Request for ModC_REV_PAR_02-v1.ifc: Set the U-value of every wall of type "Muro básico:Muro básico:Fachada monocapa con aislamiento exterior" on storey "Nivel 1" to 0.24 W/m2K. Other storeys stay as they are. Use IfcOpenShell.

First a look at what the model holds.

```python
import ifcopenshell
import ifcopenshell.util.element

model = ifcopenshell.open("ModC_REV_PAR_02-v1.ifc")
print(model.schema)
storey = next(s for s in model.by_type("IfcBuildingStorey") if s.Name == "Nivel 1")
walls = [e for e in ifcopenshell.util.element.get_decomposition(storey) if e.is_a("IfcWall")]
seen = {}
for e in walls:
    element_type = ifcopenshell.util.element.get_type(e)
    key = (element_type.Name if element_type != e and element_type else None, ifcopenshell.util.element.get_pset(e, "Pset_WallCommon", "ThermalTransmittance"))
    seen[key] = seen.get(key, 0) + 1
for (name, value), count in sorted(seen.items(), key=str):
    print(count, "x", name, "|", value)
```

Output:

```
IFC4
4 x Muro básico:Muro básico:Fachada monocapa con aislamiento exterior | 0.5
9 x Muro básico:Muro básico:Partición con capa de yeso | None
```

```python
import ifcopenshell
import ifcopenshell.api.pset
import ifcopenshell.util.element

model = ifcopenshell.open("ModC_REV_PAR_02-v1.ifc")

storey = next(s for s in model.by_type("IfcBuildingStorey") if s.Name == "Nivel 1")
walls = [e for e in ifcopenshell.util.element.get_decomposition(storey) if e.is_a("IfcWall")]

count = 0
for e in walls:
    element_type = ifcopenshell.util.element.get_type(e)
    if element_type in (None, e) or element_type.Name != "Muro básico:Muro básico:Fachada monocapa con aislamiento exterior":
        continue
    # add_pset returns the element's existing set when there is one.
    pset = ifcopenshell.api.pset.add_pset(model, product=e, name="Pset_WallCommon")
    ifcopenshell.api.pset.edit_pset(model, pset=pset, properties={"ThermalTransmittance": 0.24})
    count += 1

print(count, "walls updated")

model.write("ModC_REV_PAR_02-v1-out.ifc")
```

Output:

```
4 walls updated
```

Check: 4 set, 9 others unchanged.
